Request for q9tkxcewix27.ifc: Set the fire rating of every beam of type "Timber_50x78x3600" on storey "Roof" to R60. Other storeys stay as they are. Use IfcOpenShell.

First a look at what the model holds.

```python
import ifcopenshell
import ifcopenshell.util.element

model = ifcopenshell.open("q9tkxcewix27.ifc")
print(model.schema)
storey = next(s for s in model.by_type("IfcBuildingStorey") if s.Name == "Roof")
beams = [e for e in ifcopenshell.util.element.get_decomposition(storey) if e.is_a("IfcBeam")]
seen = {}
for e in beams:
    element_type = ifcopenshell.util.element.get_type(e)
    key = (element_type.Name if element_type != e and element_type else None, ifcopenshell.util.element.get_pset(e, "Pset_BeamCommon", "FireRating"))
    seen[key] = seen.get(key, 0) + 1
for (name, value), count in sorted(seen.items(), key=str):
    print(count, "x", name, "|", value)
```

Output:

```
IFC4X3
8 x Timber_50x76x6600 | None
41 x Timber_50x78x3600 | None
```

```python
import ifcopenshell
import ifcopenshell.api.pset
import ifcopenshell.util.element

model = ifcopenshell.open("q9tkxcewix27.ifc")

storey = next(s for s in model.by_type("IfcBuildingStorey") if s.Name == "Roof")
beams = [e for e in ifcopenshell.util.element.get_decomposition(storey) if e.is_a("IfcBeam")]

count = 0
for e in beams:
    element_type = ifcopenshell.util.element.get_type(e)
    if element_type in (None, e) or element_type.Name != "Timber_50x78x3600":
        continue
    # add_pset returns the element's existing set when there is one.
    pset = ifcopenshell.api.pset.add_pset(model, product=e, name="Pset_BeamCommon")
    ifcopenshell.api.pset.edit_pset(model, pset=pset, properties={"FireRating": "R60"})
    count += 1

print(count, "beams updated")

model.write("q9tkxcewix27_edited.ifc")
```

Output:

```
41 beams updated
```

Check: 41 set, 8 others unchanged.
